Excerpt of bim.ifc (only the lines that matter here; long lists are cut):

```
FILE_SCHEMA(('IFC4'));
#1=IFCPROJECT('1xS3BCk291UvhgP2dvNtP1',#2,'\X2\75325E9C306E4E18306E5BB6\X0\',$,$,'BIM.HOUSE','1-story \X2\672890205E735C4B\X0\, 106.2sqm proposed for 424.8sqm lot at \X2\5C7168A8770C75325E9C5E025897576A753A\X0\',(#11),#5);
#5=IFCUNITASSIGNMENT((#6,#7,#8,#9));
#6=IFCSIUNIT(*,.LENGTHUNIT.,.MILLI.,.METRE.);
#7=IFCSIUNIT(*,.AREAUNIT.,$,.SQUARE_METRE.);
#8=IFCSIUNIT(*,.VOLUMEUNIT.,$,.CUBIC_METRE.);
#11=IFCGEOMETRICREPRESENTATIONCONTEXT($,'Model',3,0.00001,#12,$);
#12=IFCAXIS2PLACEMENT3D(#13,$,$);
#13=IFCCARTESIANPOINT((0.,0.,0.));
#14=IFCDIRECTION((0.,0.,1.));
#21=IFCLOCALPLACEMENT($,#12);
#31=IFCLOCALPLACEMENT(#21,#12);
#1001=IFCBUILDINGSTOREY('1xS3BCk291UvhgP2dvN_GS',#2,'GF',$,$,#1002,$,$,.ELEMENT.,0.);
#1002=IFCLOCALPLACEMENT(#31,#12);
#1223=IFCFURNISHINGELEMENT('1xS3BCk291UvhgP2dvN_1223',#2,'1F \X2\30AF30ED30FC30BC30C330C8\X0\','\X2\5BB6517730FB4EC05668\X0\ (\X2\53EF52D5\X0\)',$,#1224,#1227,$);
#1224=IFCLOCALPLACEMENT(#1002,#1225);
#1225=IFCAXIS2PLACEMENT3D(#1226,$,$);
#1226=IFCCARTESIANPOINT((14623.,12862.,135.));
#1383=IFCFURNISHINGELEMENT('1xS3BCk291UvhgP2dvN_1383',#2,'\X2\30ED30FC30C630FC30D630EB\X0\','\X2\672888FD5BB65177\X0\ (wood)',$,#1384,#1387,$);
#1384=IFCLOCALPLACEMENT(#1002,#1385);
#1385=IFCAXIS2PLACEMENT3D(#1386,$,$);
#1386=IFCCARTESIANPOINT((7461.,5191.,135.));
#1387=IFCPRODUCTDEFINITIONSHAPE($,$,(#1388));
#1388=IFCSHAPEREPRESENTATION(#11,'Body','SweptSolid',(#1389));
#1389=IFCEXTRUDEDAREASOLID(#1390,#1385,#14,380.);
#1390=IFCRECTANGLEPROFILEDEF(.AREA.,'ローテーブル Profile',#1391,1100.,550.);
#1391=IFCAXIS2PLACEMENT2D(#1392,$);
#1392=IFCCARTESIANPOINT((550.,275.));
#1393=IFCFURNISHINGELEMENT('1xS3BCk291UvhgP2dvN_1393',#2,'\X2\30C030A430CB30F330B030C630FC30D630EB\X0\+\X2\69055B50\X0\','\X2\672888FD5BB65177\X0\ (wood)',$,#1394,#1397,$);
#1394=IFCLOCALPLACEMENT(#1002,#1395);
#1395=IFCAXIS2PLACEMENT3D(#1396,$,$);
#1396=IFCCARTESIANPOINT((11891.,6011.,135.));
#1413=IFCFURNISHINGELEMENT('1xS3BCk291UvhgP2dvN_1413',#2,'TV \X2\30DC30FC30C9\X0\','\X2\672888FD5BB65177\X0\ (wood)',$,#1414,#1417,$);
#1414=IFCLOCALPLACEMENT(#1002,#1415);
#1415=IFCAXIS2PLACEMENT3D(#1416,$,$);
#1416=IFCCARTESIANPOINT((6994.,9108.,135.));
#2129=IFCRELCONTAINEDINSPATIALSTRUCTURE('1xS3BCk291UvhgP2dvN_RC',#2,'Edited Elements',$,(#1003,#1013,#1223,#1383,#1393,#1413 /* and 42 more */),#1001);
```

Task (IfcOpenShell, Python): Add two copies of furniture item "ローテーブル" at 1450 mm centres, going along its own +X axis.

```python
import ifcopenshell
import ifcopenshell.api.geometry
import ifcopenshell.api.root
import ifcopenshell.util.element
import ifcopenshell.util.placement
import ifcopenshell.util.unit

model = ifcopenshell.open("bim.ifc")
unit_scale = ifcopenshell.util.unit.calculate_unit_scale(model)


def reuse_history(source, copy):
    """copy_class also copies each property set's owner history, people and application; keep the originals."""
    for rel in copy.IsDefinedBy:
        if rel.is_a("IfcRelDefinesByProperties") and (history := rel.RelatingPropertyDefinition.OwnerHistory):
            rel.RelatingPropertyDefinition.OwnerHistory = source.OwnerHistory
            ifcopenshell.util.element.remove_deep2(model, history)


source = model.by_guid("1xS3BCk291UvhgP2dvN_1383")
base = ifcopenshell.util.placement.get_local_placement(source.ObjectPlacement)
step = base[:3, 0] * 1.45 / unit_scale

for i in range(1, 3):
    copy = ifcopenshell.api.root.copy_class(model, product=source)
    copy.Representation = ifcopenshell.util.element.copy_deep(
        model, source.Representation, exclude=["IfcGeometricRepresentationContext", "IfcRepresentationMap"]
    )
    reuse_history(source, copy)
    matrix = base.copy()
    matrix[:3, 3] += i * step
    print("added at", matrix[:3, 3].round(3) + 0.0)
    ifcopenshell.api.geometry.edit_object_placement(model, product=copy, matrix=matrix, is_si=False)

model.write("bim-out.ifc")
```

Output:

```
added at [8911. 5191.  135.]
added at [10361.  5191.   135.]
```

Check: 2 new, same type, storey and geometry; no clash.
